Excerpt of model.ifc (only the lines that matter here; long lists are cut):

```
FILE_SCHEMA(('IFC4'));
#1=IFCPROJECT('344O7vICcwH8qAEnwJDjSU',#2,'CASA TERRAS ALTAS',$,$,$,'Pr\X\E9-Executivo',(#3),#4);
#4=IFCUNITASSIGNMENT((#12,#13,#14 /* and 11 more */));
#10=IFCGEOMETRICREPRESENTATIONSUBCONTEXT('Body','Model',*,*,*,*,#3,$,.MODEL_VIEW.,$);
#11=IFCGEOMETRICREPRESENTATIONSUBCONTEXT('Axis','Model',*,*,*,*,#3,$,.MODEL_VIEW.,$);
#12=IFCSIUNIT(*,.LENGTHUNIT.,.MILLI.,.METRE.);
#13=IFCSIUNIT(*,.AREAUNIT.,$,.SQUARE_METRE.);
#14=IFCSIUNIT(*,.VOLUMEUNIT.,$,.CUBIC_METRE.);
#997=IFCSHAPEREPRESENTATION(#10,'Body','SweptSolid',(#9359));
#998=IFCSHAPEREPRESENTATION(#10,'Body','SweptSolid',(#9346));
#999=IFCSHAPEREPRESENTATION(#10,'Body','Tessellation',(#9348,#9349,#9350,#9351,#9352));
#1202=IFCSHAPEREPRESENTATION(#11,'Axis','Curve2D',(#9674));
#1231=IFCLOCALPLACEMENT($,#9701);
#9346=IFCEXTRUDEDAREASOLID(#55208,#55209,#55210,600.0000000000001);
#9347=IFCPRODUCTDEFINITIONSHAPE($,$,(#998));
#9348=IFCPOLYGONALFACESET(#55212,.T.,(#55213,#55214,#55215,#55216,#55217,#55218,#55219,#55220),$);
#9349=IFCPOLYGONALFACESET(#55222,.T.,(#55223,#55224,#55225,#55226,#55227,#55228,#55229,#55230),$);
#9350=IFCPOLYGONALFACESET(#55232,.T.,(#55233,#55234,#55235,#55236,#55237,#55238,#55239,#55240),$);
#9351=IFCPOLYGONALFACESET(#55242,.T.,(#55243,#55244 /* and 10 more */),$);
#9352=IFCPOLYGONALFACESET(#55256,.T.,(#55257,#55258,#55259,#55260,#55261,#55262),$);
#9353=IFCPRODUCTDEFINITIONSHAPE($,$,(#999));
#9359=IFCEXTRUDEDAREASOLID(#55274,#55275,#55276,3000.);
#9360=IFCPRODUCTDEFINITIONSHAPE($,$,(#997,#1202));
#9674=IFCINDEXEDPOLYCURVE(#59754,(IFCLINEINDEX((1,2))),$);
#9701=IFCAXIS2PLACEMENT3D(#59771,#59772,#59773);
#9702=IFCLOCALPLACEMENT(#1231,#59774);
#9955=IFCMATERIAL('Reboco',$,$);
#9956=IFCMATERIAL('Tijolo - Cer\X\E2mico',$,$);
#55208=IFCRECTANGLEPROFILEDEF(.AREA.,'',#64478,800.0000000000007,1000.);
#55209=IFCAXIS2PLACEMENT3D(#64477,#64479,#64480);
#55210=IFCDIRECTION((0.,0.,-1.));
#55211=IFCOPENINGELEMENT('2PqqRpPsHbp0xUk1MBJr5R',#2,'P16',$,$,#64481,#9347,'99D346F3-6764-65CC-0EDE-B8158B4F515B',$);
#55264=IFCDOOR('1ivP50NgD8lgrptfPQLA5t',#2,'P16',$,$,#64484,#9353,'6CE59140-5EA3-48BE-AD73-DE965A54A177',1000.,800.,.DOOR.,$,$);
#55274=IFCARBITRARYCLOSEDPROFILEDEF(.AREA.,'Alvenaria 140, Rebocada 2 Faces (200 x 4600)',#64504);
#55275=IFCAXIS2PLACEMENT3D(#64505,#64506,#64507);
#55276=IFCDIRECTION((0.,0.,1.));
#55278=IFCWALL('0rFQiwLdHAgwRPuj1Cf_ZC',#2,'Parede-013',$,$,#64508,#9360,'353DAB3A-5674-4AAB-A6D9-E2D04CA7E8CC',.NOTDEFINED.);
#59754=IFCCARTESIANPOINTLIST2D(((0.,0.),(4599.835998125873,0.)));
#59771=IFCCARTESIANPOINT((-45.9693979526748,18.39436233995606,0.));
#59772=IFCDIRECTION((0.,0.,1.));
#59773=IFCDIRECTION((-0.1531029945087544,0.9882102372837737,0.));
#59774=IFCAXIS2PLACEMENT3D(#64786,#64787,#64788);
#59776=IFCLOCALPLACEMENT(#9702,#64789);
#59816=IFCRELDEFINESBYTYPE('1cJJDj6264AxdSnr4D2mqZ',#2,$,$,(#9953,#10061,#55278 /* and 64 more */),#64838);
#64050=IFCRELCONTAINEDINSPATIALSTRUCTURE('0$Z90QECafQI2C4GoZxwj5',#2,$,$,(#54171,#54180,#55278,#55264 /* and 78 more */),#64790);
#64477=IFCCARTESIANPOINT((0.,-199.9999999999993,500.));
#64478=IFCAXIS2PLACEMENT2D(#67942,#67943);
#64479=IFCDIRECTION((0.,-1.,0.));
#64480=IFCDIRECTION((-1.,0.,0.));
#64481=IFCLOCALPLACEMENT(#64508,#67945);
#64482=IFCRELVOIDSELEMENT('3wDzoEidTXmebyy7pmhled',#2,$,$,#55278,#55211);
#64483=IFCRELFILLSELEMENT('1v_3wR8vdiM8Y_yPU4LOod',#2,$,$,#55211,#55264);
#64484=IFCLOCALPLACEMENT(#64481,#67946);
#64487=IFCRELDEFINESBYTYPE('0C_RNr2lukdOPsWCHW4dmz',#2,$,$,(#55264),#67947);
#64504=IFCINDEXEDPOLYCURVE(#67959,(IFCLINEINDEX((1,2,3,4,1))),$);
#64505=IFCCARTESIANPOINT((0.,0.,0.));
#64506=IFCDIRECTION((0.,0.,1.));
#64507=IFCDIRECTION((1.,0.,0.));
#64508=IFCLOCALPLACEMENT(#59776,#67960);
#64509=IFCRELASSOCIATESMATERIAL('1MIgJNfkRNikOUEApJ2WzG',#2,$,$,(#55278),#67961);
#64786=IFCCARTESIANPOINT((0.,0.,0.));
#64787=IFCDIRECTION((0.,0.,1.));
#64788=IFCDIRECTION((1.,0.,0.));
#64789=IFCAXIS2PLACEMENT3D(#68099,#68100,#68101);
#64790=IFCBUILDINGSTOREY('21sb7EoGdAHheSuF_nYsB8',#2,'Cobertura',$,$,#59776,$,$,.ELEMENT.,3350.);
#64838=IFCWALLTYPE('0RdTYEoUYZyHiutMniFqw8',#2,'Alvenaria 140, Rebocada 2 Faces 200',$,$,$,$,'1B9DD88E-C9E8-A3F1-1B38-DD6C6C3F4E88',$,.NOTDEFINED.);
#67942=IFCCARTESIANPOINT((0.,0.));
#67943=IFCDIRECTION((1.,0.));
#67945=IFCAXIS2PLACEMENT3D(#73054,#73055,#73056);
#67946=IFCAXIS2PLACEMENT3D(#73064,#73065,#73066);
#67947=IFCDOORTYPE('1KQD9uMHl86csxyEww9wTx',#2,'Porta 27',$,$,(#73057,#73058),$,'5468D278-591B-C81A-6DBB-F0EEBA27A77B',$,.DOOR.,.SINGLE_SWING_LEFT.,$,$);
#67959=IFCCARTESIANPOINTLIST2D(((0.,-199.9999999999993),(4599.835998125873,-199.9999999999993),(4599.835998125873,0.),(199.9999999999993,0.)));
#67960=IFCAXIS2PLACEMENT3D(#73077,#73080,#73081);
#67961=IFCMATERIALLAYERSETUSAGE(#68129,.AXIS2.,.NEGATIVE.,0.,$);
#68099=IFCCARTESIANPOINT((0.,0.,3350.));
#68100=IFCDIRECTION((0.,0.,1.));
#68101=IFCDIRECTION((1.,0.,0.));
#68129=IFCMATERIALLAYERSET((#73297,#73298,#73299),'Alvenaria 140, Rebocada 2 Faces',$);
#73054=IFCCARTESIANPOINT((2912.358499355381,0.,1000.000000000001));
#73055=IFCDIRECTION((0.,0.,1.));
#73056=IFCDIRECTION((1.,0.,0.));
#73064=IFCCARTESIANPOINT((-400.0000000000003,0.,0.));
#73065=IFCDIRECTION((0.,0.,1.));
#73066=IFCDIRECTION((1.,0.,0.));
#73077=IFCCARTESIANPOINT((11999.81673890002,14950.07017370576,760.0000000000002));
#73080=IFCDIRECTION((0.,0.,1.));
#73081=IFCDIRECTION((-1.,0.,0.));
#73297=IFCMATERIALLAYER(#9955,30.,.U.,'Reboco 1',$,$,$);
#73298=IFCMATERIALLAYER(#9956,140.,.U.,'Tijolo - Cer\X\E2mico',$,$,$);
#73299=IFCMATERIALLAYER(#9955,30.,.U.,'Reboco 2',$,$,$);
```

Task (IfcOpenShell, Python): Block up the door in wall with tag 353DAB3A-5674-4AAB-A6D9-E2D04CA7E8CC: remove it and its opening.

```python
import ifcopenshell
import ifcopenshell.api.feature
import ifcopenshell.api.root
import ifcopenshell.geom
import ifcopenshell.util.shape

model = ifcopenshell.open("model.ifc")
settings = ifcopenshell.geom.settings()


def volume(element):
    """Net volume in cubic metres, openings subtracted."""
    shape = ifcopenshell.geom.create_shape(settings, element)
    return ifcopenshell.util.shape.get_volume(shape.geometry)


door = model.by_guid("1ivP50NgD8lgrptfPQLA5t")
opening = door.FillsVoids[0].RelatingOpeningElement
wall = opening.VoidsElements[0].RelatingBuildingElement
before = volume(wall)

ifcopenshell.api.root.remove_product(model, product=door)
ifcopenshell.api.feature.remove_feature(model, feature=opening)

after = volume(wall)

print(f"wall volume {before:.3f} -> {after:.3f} m3")

model.write("model_updated.ifc")
```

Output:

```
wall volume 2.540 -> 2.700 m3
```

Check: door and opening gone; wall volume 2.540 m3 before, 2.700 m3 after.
